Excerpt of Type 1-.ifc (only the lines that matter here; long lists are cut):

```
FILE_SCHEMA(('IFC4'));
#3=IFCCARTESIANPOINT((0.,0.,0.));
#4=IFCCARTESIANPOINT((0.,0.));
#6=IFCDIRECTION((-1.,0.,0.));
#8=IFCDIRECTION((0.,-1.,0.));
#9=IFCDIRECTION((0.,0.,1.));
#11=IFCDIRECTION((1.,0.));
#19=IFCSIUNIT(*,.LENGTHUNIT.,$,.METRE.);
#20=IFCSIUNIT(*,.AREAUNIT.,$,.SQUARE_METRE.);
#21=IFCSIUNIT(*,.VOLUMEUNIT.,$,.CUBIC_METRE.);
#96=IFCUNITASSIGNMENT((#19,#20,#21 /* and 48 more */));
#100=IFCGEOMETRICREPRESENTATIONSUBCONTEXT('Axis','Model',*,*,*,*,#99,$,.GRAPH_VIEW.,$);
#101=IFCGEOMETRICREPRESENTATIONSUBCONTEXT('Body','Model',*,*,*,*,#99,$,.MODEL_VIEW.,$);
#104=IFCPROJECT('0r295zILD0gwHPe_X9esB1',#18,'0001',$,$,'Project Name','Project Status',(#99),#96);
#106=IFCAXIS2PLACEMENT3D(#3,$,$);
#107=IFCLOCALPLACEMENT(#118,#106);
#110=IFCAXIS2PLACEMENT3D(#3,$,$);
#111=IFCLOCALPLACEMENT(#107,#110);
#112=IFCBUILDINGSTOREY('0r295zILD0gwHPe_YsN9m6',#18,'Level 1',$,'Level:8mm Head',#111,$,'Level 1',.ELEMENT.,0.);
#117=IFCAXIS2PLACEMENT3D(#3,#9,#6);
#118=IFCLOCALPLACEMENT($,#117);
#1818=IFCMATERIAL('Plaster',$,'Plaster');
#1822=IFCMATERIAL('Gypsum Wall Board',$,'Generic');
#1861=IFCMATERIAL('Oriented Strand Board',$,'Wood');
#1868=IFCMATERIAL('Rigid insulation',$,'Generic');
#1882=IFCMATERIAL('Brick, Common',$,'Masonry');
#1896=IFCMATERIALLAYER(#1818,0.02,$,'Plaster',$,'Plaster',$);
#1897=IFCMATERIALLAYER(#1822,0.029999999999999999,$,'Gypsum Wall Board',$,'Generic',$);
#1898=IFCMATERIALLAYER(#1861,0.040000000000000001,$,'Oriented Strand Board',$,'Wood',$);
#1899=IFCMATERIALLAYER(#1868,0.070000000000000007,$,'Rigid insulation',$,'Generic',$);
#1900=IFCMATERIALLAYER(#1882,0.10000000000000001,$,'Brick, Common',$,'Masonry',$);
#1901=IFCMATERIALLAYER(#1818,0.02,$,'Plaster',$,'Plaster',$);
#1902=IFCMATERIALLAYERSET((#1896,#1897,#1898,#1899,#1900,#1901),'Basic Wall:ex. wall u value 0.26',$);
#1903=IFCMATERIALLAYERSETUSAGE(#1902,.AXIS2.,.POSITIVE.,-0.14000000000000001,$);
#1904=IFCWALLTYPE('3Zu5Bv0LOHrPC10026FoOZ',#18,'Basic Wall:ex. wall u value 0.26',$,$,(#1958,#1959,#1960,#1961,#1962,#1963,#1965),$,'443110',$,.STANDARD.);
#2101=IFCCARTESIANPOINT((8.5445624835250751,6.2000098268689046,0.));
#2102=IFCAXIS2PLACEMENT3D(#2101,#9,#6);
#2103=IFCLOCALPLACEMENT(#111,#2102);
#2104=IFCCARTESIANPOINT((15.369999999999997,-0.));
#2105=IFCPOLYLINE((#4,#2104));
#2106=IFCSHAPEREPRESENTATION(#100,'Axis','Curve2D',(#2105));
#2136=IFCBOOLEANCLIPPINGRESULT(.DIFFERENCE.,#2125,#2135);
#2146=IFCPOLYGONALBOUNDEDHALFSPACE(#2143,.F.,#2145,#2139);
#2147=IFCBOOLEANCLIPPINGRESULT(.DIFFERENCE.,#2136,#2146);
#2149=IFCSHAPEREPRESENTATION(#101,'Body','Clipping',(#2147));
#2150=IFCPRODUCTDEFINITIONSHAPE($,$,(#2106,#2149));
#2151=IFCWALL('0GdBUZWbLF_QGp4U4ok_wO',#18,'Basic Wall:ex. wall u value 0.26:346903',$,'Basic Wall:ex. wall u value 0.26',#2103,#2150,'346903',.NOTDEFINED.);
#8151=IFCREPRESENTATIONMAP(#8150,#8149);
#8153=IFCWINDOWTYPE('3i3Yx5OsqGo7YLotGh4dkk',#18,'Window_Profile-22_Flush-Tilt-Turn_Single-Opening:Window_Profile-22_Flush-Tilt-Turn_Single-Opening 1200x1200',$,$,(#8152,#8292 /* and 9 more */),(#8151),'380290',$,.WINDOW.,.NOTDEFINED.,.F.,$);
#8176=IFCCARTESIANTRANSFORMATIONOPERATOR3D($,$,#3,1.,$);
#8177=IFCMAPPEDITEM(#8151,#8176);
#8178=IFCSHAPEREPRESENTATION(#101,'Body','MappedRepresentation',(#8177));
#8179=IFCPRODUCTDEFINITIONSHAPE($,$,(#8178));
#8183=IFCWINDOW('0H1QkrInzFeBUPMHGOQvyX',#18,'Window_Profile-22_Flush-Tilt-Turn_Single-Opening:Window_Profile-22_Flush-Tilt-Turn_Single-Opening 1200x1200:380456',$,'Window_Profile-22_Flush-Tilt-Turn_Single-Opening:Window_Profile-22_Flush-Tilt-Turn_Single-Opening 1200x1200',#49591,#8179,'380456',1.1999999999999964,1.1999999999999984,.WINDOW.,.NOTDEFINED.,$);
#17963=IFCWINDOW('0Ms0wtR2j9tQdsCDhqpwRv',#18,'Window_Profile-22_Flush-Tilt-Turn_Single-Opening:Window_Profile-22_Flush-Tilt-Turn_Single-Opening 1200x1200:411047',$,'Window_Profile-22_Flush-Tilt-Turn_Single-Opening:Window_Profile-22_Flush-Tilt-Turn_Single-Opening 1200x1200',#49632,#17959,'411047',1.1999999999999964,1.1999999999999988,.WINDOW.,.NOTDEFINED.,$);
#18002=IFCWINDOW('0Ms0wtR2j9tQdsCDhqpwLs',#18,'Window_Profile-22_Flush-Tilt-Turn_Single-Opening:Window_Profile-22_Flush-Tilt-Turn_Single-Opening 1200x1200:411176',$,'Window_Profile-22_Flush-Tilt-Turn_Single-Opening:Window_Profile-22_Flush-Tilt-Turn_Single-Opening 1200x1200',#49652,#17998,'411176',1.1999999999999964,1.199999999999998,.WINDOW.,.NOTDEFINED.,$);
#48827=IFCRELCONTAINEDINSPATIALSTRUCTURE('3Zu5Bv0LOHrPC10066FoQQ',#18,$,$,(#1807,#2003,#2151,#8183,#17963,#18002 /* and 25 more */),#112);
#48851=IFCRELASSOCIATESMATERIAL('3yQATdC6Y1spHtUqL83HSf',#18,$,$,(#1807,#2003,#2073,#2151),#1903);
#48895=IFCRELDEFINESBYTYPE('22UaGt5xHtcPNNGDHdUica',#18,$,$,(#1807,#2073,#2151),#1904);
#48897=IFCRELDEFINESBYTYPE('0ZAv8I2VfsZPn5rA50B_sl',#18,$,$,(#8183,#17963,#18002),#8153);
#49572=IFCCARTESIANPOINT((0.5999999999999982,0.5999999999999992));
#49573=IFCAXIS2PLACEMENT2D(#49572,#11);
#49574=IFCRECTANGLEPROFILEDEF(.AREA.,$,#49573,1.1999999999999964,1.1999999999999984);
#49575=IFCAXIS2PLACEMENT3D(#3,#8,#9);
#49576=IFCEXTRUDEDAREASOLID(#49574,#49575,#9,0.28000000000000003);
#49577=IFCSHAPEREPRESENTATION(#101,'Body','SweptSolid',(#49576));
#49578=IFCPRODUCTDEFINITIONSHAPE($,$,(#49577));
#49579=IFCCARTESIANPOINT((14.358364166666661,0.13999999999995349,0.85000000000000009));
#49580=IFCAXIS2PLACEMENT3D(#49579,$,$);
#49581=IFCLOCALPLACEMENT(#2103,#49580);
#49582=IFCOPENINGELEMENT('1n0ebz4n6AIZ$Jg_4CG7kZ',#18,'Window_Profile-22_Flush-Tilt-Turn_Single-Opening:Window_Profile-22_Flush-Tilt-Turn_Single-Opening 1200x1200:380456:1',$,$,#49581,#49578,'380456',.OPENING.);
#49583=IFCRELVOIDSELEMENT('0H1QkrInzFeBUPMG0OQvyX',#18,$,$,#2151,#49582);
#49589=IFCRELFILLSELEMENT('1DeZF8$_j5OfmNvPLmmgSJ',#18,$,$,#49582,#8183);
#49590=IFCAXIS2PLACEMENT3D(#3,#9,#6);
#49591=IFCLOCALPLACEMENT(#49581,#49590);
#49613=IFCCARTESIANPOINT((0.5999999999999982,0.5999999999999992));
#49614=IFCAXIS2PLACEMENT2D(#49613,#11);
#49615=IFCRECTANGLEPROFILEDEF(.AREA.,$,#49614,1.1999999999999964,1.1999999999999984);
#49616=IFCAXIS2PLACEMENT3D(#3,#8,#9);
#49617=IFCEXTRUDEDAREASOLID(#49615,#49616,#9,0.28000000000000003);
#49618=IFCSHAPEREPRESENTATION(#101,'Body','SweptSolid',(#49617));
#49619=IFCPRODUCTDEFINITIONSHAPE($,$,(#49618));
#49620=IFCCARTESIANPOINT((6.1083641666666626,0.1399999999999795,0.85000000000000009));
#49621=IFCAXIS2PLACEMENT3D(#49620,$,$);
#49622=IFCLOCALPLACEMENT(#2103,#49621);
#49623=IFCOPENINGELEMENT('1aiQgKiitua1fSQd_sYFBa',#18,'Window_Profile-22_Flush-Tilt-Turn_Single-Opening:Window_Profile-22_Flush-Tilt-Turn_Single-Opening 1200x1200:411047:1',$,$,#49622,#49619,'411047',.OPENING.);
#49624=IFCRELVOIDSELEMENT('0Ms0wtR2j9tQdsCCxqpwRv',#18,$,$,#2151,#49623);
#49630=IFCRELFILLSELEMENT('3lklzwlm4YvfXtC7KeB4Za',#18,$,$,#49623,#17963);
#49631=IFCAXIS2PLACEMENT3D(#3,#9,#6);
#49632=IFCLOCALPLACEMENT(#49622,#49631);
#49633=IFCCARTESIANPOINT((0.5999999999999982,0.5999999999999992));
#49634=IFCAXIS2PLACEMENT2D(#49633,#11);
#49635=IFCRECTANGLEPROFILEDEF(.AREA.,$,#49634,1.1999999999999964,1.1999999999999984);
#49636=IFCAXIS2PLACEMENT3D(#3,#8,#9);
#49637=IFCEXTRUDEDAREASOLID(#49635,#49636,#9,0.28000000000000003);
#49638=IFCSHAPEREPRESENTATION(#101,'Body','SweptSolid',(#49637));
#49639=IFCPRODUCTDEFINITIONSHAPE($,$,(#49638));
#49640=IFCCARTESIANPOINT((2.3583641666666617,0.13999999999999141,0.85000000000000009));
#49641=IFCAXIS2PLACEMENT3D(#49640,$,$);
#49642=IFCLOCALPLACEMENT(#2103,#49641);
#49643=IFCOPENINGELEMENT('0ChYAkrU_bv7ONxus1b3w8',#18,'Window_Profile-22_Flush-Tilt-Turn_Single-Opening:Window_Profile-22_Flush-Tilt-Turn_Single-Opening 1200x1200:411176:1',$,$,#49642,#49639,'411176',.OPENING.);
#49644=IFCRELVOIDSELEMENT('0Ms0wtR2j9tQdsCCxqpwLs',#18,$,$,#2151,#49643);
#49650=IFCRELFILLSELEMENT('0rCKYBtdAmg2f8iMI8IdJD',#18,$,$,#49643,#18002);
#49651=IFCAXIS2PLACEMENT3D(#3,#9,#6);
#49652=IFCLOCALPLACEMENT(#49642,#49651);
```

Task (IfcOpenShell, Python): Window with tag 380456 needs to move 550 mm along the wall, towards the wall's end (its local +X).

```python
import ifcopenshell
import ifcopenshell.api.geometry
import ifcopenshell.util.placement
import ifcopenshell.util.unit

model = ifcopenshell.open("Type 1-.ifc")
unit_scale = ifcopenshell.util.unit.calculate_unit_scale(model)

window = model.by_id(8183)
opening = window.FillsVoids[0].RelatingOpeningElement
wall = opening.VoidsElements[0].RelatingBuildingElement

wall_matrix = ifcopenshell.util.placement.get_local_placement(wall.ObjectPlacement)
shift = wall_matrix[:3, 0] * 0.55 / unit_scale
before = ifcopenshell.util.placement.get_local_placement(window.ObjectPlacement)[:3, 3].copy()

# The window is placed relative to its opening, so it follows when the opening moves.
matrix = ifcopenshell.util.placement.get_local_placement(opening.ObjectPlacement)
matrix[:3, 3] += shift
ifcopenshell.api.geometry.edit_object_placement(
    model, product=opening, matrix=matrix, is_si=False, should_transform_children=True
)

after = ifcopenshell.util.placement.get_local_placement(window.ObjectPlacement)[:3, 3]
print("window moved by", (after - before).round(3) + 0.0)

model.write("Type 1-_edited.ifc")
```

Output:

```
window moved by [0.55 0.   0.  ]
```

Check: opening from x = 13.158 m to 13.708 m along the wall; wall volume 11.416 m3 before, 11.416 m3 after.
